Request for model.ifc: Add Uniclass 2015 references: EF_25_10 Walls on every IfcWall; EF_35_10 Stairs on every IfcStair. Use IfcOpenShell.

First a look at what the model holds.

```python
import ifcopenshell

model = ifcopenshell.open("model.ifc")
print(model.schema)
print("classifications:", [c.Name for c in model.by_type("IfcClassification")])
for ifc_class in ("IfcDoor", "IfcRoof", "IfcStair", "IfcWall", "IfcWindow"):
    print(ifc_class, len(model.by_type(ifc_class)))
```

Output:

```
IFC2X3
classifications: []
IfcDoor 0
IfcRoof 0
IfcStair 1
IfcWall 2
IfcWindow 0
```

```python
import ifcopenshell
import ifcopenshell.api.classification

model = ifcopenshell.open("model.ifc")

# IFC2X3 requires Source and Edition and has no link from the project to the system.
system = model.create_entity("IfcClassification", Source="NBS", Edition="2015", Name="Uniclass 2015")

codes = {
    "IfcWall": ("EF_25_10", "Walls"),
    "IfcStair": ("EF_35_10", "Stairs"),
}
for ifc_class, (code, name) in codes.items():
    products = model.by_type(ifc_class)
    ifcopenshell.api.classification.add_reference(
        model, products=products, classification=system, identification=code, name=name
    )
    print(code, len(products))

model.write("model_rev.ifc")
```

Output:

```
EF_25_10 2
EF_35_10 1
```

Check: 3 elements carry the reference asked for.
